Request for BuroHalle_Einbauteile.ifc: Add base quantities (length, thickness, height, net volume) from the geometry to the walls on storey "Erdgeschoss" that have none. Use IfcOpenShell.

First a look at what the model holds.

```python
import ifcopenshell
import ifcopenshell.util.element
import ifcopenshell.util.unit

model = ifcopenshell.open("BuroHalle_Einbauteile.ifc")
print(model.schema)
for unit_type in ("LENGTHUNIT", "AREAUNIT", "VOLUMEUNIT"):
    print(unit_type, ifcopenshell.util.unit.calculate_unit_scale(model, unit_type))
storey = next(s for s in model.by_type("IfcBuildingStorey") if s.Name == "Erdgeschoss")
walls = [e for e in ifcopenshell.util.element.get_decomposition(storey) if e.is_a("IfcWall")]
for e in sorted(walls, key=lambda e: e.id()):
    print(e.id(), e.is_a(), e.Name, list(ifcopenshell.util.element.get_psets(e, qtos_only=True)), sep=" | ")
```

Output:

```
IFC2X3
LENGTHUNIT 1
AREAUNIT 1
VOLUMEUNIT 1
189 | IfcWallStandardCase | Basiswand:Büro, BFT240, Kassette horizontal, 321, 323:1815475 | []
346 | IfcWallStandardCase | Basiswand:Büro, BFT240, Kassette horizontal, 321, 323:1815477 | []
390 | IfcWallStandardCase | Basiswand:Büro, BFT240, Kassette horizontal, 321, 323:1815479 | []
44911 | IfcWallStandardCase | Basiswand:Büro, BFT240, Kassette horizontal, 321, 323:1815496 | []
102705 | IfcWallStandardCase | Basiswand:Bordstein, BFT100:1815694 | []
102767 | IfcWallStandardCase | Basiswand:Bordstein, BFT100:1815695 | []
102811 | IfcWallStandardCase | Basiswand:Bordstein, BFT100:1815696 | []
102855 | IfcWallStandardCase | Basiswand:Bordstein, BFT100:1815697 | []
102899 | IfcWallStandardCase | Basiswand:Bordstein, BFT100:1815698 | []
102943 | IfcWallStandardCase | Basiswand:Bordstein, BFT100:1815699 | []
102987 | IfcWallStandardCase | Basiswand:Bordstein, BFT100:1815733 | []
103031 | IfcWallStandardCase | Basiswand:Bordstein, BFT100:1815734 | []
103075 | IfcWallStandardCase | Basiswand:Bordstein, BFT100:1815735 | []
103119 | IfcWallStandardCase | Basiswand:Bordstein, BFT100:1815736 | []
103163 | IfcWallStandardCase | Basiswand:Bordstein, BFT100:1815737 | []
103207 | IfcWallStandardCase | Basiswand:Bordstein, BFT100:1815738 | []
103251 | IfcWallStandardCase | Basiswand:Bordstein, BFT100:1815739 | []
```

```python
import ifcopenshell
import ifcopenshell.api.pset
import ifcopenshell.geom
import ifcopenshell.util.element
import ifcopenshell.util.shape
import ifcopenshell.util.unit

model = ifcopenshell.open("BuroHalle_Einbauteile.ifc")
unit_scale = ifcopenshell.util.unit.calculate_unit_scale(model)
volume_scale = ifcopenshell.util.unit.calculate_unit_scale(model, "VOLUMEUNIT")
settings = ifcopenshell.geom.settings()

storey = next(s for s in model.by_type("IfcBuildingStorey") if s.Name == "Erdgeschoss")
walls = [e for e in ifcopenshell.util.element.get_decomposition(storey) if e.is_a("IfcWall")]

for e in sorted(walls, key=lambda e: e.id()):
    if ifcopenshell.util.element.get_psets(e, qtos_only=True, should_inherit=False):
        continue
    # Geometry comes back in metres, in the element's own axes.
    shape = ifcopenshell.geom.create_shape(settings, e)
    values = {
        "Length": ifcopenshell.util.shape.get_x(shape.geometry) / unit_scale,
        "Width": ifcopenshell.util.shape.get_y(shape.geometry) / unit_scale,
        "Height": ifcopenshell.util.shape.get_z(shape.geometry) / unit_scale,
        "NetVolume": ifcopenshell.util.shape.get_volume(shape.geometry) / volume_scale,
    }
    qto = ifcopenshell.api.pset.add_qto(model, product=e, name="BaseQuantities")
    ifcopenshell.api.pset.edit_qto(model, qto=qto, properties=values)
    print(e.id(), {k: round(v, 3) for k, v in values.items()})

model.write("BuroHalle_Einbauteile_edited.ifc")
```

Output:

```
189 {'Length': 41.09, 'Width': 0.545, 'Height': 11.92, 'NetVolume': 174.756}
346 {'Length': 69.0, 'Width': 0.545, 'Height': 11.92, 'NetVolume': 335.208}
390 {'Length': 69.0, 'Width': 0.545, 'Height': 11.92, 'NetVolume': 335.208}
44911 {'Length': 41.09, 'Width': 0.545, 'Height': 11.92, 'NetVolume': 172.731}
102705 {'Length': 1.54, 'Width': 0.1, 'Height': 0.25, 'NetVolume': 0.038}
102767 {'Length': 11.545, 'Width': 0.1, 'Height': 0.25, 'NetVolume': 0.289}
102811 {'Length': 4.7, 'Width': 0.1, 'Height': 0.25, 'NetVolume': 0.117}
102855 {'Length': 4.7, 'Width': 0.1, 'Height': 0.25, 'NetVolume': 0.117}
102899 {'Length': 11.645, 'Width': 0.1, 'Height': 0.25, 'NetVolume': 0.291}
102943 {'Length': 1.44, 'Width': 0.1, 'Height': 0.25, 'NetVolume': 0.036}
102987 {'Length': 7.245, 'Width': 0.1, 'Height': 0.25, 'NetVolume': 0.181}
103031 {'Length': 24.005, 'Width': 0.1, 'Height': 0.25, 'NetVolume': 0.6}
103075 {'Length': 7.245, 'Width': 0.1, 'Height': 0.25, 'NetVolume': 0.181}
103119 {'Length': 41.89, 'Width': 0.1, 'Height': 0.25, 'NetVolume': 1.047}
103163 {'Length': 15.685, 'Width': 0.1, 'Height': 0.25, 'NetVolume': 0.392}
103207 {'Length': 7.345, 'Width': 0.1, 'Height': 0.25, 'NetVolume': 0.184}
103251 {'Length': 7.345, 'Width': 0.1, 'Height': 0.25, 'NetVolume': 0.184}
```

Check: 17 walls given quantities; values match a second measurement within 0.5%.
